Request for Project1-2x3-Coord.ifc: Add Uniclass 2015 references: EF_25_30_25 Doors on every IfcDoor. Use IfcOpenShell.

First a look at what the model holds.

```python
import ifcopenshell

model = ifcopenshell.open("Project1-2x3-Coord.ifc")
print(model.schema)
print("classifications:", [c.Name for c in model.by_type("IfcClassification")])
for ifc_class in ("IfcDoor", "IfcRoof", "IfcStair", "IfcWall", "IfcWindow"):
    print(ifc_class, len(model.by_type(ifc_class)))
```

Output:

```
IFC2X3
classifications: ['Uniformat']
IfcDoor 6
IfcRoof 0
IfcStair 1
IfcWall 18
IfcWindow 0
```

```python
import ifcopenshell
import ifcopenshell.api.classification

model = ifcopenshell.open("Project1-2x3-Coord.ifc")

# IFC2X3 requires Source and Edition and has no link from the project to the system.
system = model.create_entity("IfcClassification", Source="NBS", Edition="2015", Name="Uniclass 2015")

codes = {
    "IfcDoor": ("EF_25_30_25", "Doors"),
}
for ifc_class, (code, name) in codes.items():
    products = model.by_type(ifc_class)
    ifcopenshell.api.classification.add_reference(
        model, products=products, classification=system, identification=code, name=name
    )
    print(code, len(products))

model.write("Project1-2x3-Coord_rev.ifc")
```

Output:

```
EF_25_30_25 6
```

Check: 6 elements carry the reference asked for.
